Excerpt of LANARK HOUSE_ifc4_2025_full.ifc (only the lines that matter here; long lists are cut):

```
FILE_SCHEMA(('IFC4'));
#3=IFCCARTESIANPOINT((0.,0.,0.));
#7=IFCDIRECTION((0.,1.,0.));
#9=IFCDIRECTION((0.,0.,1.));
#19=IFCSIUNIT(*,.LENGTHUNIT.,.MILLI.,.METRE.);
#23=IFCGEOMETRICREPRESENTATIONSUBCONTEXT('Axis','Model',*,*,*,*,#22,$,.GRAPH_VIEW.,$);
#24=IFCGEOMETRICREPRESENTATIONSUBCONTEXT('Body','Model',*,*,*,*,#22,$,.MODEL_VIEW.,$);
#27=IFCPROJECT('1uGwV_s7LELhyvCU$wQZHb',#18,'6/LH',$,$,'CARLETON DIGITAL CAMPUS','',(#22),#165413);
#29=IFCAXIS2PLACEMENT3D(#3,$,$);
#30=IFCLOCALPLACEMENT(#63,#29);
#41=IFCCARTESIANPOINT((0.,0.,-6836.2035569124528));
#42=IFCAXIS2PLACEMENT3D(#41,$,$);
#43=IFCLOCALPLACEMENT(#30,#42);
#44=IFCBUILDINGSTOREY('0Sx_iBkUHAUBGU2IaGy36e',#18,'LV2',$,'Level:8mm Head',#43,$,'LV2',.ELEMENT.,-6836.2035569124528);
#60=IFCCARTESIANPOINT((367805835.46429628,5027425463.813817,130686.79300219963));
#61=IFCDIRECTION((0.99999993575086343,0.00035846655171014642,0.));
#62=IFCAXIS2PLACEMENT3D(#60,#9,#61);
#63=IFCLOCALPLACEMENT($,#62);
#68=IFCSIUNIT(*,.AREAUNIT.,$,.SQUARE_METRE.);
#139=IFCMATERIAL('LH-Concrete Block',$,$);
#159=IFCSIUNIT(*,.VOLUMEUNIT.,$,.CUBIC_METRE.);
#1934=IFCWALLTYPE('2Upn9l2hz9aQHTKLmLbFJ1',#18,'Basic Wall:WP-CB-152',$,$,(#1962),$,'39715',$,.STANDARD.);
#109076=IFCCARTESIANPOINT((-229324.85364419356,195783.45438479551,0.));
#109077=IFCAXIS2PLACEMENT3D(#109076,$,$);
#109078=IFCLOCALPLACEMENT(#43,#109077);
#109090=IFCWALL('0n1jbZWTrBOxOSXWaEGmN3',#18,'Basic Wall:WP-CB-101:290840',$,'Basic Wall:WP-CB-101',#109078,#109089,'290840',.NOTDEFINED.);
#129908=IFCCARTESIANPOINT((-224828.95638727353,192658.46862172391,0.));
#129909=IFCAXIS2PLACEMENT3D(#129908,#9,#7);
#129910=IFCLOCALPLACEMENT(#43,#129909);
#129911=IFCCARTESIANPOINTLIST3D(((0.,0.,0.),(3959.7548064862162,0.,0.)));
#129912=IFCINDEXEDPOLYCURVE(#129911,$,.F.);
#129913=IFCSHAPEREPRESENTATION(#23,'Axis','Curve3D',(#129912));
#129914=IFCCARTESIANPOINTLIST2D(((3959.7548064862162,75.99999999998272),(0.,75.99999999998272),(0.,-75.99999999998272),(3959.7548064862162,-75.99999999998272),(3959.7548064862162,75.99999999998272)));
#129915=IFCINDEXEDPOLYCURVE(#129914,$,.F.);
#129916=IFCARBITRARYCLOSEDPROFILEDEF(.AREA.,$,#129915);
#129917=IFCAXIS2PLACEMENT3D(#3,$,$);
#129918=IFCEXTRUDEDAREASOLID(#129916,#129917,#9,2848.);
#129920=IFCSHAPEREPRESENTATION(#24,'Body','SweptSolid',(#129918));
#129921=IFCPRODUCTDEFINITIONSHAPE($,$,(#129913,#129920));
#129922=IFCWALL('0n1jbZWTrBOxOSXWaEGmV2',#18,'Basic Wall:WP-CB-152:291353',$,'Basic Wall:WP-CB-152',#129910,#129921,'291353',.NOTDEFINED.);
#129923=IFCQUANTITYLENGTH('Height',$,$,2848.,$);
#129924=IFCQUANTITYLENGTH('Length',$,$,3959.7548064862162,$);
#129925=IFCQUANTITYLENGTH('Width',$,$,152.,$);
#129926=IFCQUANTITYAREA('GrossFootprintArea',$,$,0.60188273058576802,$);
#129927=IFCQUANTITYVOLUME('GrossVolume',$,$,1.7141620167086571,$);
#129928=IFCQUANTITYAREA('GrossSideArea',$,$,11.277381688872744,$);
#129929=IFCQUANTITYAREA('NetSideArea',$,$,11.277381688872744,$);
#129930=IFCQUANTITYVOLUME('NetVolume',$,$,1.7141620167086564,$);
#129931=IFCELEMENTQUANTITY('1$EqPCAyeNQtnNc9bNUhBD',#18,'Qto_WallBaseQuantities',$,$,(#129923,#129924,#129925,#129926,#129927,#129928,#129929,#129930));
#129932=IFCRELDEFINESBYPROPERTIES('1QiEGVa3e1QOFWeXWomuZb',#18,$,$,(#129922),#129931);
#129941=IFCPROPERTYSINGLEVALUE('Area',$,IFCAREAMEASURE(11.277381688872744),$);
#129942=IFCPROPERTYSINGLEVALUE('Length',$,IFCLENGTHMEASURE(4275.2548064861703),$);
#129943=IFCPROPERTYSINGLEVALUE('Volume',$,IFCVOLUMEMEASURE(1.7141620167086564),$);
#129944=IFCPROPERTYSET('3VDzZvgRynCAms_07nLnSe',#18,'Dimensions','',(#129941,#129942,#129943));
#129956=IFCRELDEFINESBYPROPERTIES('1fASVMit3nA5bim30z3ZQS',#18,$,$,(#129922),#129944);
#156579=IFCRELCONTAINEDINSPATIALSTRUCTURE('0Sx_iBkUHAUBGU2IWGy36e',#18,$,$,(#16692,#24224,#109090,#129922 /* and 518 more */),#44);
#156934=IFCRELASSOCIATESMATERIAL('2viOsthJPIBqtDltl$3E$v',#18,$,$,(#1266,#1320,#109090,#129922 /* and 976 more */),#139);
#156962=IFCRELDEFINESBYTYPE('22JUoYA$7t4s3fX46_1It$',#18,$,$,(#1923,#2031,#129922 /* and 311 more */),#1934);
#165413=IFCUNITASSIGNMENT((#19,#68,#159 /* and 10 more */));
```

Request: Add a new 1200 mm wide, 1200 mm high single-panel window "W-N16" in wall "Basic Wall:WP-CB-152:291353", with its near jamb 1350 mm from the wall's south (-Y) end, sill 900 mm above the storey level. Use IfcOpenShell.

```python
import numpy as np
import ifcopenshell
import ifcopenshell.api.feature
import ifcopenshell.api.geometry
import ifcopenshell.api.pset
import ifcopenshell.api.root
import ifcopenshell.api.spatial
import ifcopenshell.geom
import ifcopenshell.util.element
import ifcopenshell.util.placement
import ifcopenshell.util.representation
import ifcopenshell.util.shape
import ifcopenshell.util.unit

model = ifcopenshell.open("LANARK HOUSE_ifc4_2025_full.ifc")
unit_scale = ifcopenshell.util.unit.calculate_unit_scale(model)
area_scale = ifcopenshell.util.unit.calculate_unit_scale(model, "AREAUNIT")
volume_scale = ifcopenshell.util.unit.calculate_unit_scale(model, "VOLUMEUNIT")
settings = ifcopenshell.geom.settings()


def volume(element):
    """Net volume in cubic metres, openings subtracted."""
    shape = ifcopenshell.geom.create_shape(settings, element)
    return ifcopenshell.util.shape.get_volume(shape.geometry)


wall = model.by_guid("0n1jbZWTrBOxOSXWaEGmV2")
storey = ifcopenshell.util.element.get_container(wall, ifc_class="IfcBuildingStorey")
context = ifcopenshell.util.representation.get_context(model, "Model", "Body", "MODEL_VIEW")
before = volume(wall)

width, height, from_end, sill = 1.2, 1.2, 1.35, 0.9  # metres

# The wall runs along its own X axis, and the end named is its -X end.
wall_shape = ifcopenshell.geom.create_shape(settings, wall)
x, y, z = ifcopenshell.util.shape.get_vertices(wall_shape.geometry).T
start = x.min() + from_end
face, thickness = float(y.min()), float(y.max() - y.min())
wall_matrix = ifcopenshell.util.placement.get_local_placement(wall.ObjectPlacement)
level = ifcopenshell.util.placement.get_local_placement(storey.ObjectPlacement)[2, 3]


def in_wall(x, y):
    """Placement at x, y metres in the wall's axes, at sill height."""
    matrix = wall_matrix.copy()
    matrix[:, 3] = wall_matrix @ np.array([x / unit_scale, y / unit_scale, 0.0, 1.0])
    matrix[2, 3] = level + sill / unit_scale
    return matrix


# Opening: a box that overshoots both wall faces by 50 mm.
opening = ifcopenshell.api.root.create_entity(model, ifc_class="IfcOpeningElement", predefined_type="OPENING")
box = ifcopenshell.api.geometry.add_wall_representation(
    model, context=context, length=width, height=height, thickness=thickness + 0.1
)
ifcopenshell.api.geometry.assign_representation(model, product=opening, representation=box)
ifcopenshell.api.geometry.edit_object_placement(model, product=opening, matrix=in_wall(start, face - 0.05), is_si=False)
ifcopenshell.api.feature.add_feature(model, feature=opening, element=wall)

window = ifcopenshell.api.root.create_entity(model, ifc_class="IfcWindow", name="W-N16", predefined_type="WINDOW")
window.OverallWidth, window.OverallHeight = width / unit_scale, height / unit_scale
window.PartitioningType = "SINGLE_PANEL"
body = ifcopenshell.api.geometry.add_window_representation(
    model,
    context=context,
    overall_width=window.OverallWidth,
    overall_height=window.OverallHeight,
    partition_type="SINGLE_PANEL",
)
ifcopenshell.api.geometry.assign_representation(model, product=window, representation=body)
ifcopenshell.api.spatial.assign_container(model, products=[window], relating_structure=storey)
ifcopenshell.api.feature.add_filling(model, opening=opening, element=window)

# Centre the window in the wall's thickness.
ifcopenshell.api.geometry.edit_object_placement(model, product=window, matrix=in_wall(start, face), is_si=False)
window_shape = ifcopenshell.geom.create_shape(settings, window)
depth = ifcopenshell.util.shape.get_vertices(window_shape.geometry)[:, 1]
offset = face + thickness / 2 - (depth.min() + depth.max()) / 2
ifcopenshell.api.geometry.edit_object_placement(model, product=window, matrix=in_wall(start, offset), is_si=False)

after = volume(wall)

# Update the wall's stored quantities.
qto = model.by_id(ifcopenshell.util.element.get_pset(wall, "Qto_WallBaseQuantities", should_inherit=False)["id"])
ifcopenshell.api.pset.edit_qto(model, qto=qto, properties={
    "NetSideArea": after / thickness / area_scale,
    "NetVolume": after / volume_scale,
})
pset = model.by_id(ifcopenshell.util.element.get_pset(wall, "Dimensions", should_inherit=False)["id"])
ifcopenshell.api.pset.edit_pset(model, pset=pset, properties={
    "Area": model.create_entity("IfcAreaMeasure", after / thickness / area_scale),
    "Volume": model.create_entity("IfcVolumeMeasure", after / volume_scale),
})

print(f"wall volume {before:.3f} -> {after:.3f} m3")

model.write("LANARK HOUSE_ifc4_2025_full_rev.ifc")
```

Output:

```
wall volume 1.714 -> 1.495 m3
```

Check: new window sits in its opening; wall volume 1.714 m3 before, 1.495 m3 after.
